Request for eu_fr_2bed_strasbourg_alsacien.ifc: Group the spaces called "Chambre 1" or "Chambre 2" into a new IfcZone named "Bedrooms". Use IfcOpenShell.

First a look at what the model holds.

```python
import ifcopenshell

model = ifcopenshell.open("eu_fr_2bed_strasbourg_alsacien.ifc")
print(model.schema)
seen = {}
for space in model.by_type("IfcSpace"):
    seen[space.LongName] = seen.get(space.LongName, 0) + 1
for name, count in sorted(seen.items(), key=str):
    print(count, "x", name)
print("zones:", [z.Name for z in model.by_type("IfcZone")][:20])
```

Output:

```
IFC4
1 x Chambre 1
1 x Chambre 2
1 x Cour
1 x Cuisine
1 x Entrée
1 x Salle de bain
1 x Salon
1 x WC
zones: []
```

```python
import ifcopenshell
import ifcopenshell.api.group
import ifcopenshell.api.root

model = ifcopenshell.open("eu_fr_2bed_strasbourg_alsacien.ifc")

names = {"Chambre 1", "Chambre 2"}
spaces = [s for s in model.by_type("IfcSpace") if s.LongName in names]

zone = ifcopenshell.api.root.create_entity(model, ifc_class="IfcZone", name="Bedrooms")
ifcopenshell.api.group.assign_group(model, products=spaces, group=zone)
print(len(spaces), "spaces in", zone.Name)

model.write("eu_fr_2bed_strasbourg_alsacien_edited.ifc")
```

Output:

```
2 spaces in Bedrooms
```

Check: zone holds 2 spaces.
